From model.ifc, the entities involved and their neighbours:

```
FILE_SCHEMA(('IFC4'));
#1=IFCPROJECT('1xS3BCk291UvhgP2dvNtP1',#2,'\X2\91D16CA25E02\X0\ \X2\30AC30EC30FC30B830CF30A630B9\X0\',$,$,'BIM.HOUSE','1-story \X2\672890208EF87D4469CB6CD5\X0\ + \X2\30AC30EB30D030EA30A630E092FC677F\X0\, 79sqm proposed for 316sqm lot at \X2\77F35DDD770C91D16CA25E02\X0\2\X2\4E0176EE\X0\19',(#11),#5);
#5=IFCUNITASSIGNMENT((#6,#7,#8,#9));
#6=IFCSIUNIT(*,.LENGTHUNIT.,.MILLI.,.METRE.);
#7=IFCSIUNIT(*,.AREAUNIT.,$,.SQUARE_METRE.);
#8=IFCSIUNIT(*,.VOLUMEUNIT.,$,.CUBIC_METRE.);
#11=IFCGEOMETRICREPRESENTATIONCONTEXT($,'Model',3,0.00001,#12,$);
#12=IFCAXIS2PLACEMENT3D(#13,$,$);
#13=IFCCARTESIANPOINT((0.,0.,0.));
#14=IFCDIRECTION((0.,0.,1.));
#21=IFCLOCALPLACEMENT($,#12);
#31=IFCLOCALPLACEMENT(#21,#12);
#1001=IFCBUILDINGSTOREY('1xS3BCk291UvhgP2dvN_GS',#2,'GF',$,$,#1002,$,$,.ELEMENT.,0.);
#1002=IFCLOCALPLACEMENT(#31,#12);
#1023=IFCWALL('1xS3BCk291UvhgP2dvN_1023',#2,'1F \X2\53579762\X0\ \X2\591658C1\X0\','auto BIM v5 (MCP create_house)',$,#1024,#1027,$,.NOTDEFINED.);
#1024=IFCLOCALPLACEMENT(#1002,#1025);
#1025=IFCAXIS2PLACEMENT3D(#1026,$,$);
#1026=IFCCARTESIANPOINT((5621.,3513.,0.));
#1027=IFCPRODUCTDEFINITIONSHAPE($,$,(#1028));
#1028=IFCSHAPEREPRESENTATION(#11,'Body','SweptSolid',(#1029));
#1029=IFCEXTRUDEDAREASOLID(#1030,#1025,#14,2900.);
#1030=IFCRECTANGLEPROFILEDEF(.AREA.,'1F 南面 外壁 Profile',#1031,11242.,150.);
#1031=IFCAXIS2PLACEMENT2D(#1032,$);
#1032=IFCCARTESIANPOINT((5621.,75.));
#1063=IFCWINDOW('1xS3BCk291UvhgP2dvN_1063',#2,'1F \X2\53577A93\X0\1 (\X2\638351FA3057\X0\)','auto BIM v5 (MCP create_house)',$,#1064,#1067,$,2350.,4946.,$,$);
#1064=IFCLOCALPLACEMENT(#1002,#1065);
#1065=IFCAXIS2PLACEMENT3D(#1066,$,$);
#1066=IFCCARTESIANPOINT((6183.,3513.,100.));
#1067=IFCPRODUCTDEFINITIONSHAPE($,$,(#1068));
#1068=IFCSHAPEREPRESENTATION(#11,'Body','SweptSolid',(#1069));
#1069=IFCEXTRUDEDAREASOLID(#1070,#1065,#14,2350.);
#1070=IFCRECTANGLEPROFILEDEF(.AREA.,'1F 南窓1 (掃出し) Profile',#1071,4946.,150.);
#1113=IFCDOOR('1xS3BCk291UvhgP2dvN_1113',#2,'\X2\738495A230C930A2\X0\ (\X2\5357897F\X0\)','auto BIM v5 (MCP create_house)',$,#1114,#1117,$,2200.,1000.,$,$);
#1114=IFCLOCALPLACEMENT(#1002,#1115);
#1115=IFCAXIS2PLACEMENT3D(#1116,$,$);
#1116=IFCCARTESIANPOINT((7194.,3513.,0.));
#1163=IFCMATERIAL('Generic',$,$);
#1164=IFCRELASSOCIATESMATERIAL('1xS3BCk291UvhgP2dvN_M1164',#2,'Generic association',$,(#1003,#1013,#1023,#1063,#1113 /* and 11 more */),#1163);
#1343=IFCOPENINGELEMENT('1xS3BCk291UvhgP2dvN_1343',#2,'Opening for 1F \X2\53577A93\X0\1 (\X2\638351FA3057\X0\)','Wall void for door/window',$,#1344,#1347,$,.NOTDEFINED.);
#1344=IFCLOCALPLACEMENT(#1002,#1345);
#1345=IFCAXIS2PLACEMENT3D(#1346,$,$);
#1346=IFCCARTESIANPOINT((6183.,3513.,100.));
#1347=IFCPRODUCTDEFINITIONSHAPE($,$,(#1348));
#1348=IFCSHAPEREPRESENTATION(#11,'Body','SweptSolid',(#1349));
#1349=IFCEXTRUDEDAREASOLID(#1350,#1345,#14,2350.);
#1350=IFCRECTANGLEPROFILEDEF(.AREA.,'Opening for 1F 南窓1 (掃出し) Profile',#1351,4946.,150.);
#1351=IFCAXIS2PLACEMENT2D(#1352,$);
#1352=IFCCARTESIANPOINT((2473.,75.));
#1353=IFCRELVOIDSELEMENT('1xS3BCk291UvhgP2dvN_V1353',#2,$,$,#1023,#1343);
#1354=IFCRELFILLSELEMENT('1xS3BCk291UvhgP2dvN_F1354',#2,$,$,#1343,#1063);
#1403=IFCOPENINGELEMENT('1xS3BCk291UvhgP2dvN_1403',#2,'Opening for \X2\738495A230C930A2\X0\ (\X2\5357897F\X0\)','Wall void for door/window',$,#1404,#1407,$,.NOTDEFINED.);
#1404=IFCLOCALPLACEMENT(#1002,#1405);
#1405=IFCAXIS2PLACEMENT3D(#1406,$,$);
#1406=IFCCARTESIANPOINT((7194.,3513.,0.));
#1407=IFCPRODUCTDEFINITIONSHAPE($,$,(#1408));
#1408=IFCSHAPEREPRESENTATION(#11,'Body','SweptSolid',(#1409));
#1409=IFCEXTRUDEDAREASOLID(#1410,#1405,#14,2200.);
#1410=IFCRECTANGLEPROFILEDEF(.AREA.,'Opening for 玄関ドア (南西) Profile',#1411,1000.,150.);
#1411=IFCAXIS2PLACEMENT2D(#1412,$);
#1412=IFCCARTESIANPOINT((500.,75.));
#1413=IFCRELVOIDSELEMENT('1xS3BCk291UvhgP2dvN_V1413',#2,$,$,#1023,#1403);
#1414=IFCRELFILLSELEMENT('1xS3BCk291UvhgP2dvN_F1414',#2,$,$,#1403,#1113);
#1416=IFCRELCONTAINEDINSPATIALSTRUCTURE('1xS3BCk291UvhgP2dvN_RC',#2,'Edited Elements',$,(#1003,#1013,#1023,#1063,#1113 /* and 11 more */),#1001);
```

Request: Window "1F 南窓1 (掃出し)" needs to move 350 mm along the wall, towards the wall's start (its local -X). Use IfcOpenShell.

```python
import ifcopenshell
import ifcopenshell.api.geometry
import ifcopenshell.util.placement
import ifcopenshell.util.unit

model = ifcopenshell.open("model.ifc")
unit_scale = ifcopenshell.util.unit.calculate_unit_scale(model)

window = model.by_guid("1xS3BCk291UvhgP2dvN_1063")
opening = window.FillsVoids[0].RelatingOpeningElement
wall = opening.VoidsElements[0].RelatingBuildingElement

wall_matrix = ifcopenshell.util.placement.get_local_placement(wall.ObjectPlacement)
shift = wall_matrix[:3, 0] * -0.35 / unit_scale
before = ifcopenshell.util.placement.get_local_placement(window.ObjectPlacement)[:3, 3].copy()

# The window is not placed relative to its opening, so move both.
for product in (opening, window):
    matrix = ifcopenshell.util.placement.get_local_placement(product.ObjectPlacement)
    matrix[:3, 3] += shift
    ifcopenshell.api.geometry.edit_object_placement(model, product=product, matrix=matrix, is_si=False)

after = ifcopenshell.util.placement.get_local_placement(window.ObjectPlacement)[:3, 3]
print("window moved by", (after - before).round(3) + 0.0)

model.write("model_updated.ifc")
```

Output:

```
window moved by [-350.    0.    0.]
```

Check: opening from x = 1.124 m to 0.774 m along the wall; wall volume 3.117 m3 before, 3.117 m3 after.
